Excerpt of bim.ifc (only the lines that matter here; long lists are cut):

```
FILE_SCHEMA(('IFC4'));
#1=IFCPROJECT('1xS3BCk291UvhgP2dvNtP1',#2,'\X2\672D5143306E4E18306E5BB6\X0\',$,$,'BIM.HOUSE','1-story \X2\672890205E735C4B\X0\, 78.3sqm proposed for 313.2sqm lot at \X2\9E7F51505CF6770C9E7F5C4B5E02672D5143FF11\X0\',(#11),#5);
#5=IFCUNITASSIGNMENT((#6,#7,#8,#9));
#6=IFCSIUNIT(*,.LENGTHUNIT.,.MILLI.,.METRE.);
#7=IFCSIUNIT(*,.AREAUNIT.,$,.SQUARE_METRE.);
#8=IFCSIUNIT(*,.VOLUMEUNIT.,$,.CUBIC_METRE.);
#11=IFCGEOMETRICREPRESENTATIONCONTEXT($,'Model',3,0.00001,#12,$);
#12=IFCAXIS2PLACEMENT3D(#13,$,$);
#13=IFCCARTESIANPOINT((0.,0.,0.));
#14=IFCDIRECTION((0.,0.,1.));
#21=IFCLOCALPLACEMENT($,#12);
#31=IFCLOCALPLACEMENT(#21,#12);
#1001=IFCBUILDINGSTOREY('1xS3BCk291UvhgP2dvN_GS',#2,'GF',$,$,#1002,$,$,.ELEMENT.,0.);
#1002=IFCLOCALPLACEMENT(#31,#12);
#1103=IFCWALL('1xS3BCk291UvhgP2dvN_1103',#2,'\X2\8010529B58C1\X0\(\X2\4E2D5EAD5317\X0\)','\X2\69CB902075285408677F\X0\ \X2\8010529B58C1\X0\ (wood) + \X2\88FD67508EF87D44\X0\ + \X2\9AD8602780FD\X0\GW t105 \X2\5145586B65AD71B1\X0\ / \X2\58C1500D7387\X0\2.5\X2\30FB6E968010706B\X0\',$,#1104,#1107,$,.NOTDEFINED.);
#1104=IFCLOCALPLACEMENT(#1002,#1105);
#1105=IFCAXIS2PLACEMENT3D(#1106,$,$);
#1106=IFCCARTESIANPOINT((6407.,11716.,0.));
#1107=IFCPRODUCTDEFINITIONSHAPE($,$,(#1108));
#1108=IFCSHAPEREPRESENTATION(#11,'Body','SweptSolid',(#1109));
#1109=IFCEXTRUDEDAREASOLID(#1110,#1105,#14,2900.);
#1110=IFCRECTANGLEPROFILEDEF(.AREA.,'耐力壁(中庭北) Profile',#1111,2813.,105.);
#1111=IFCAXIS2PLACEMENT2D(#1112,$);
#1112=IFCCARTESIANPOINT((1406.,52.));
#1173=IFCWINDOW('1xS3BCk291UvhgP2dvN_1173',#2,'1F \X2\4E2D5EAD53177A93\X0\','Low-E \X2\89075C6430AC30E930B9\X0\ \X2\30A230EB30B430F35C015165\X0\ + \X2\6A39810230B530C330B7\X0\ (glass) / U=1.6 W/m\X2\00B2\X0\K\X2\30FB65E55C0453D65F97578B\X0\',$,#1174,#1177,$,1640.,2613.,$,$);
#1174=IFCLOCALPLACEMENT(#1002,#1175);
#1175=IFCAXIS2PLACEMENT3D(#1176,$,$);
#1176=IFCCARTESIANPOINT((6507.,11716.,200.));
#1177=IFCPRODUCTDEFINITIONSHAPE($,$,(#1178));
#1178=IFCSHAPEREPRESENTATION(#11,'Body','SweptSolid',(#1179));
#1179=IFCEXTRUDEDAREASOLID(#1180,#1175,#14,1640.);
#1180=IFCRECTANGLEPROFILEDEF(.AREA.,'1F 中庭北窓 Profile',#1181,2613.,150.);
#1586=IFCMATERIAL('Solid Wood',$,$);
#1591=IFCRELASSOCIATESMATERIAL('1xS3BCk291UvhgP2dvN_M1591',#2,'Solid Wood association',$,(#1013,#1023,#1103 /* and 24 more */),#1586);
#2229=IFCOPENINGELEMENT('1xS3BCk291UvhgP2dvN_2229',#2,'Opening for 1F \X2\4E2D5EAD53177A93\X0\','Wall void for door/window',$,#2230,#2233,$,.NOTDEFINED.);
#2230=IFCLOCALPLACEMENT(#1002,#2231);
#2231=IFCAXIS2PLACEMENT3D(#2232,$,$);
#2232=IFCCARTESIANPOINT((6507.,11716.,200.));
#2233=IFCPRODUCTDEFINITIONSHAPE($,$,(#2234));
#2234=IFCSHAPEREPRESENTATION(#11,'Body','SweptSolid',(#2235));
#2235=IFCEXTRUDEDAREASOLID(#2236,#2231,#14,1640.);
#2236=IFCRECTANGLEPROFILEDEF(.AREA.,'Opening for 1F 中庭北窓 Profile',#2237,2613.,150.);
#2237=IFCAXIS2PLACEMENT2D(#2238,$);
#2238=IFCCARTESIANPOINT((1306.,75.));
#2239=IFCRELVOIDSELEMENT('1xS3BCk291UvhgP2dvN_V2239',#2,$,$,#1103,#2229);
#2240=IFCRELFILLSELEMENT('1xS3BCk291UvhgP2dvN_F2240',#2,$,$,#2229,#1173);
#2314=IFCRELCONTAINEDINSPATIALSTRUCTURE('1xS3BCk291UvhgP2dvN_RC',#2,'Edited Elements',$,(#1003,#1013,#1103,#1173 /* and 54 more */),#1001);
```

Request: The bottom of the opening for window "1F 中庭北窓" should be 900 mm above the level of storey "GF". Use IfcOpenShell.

```python
import numpy as np
import ifcopenshell
import ifcopenshell.api.geometry
import ifcopenshell.geom
import ifcopenshell.util.element
import ifcopenshell.util.placement
import ifcopenshell.util.shape
import ifcopenshell.util.unit

model = ifcopenshell.open("bim.ifc")
unit_scale = ifcopenshell.util.unit.calculate_unit_scale(model)

window = model.by_guid("1xS3BCk291UvhgP2dvN_1173")
opening = window.FillsVoids[0].RelatingOpeningElement
storey = ifcopenshell.util.element.get_container(window, ifc_class="IfcBuildingStorey")
level = ifcopenshell.util.placement.get_local_placement(storey.ObjectPlacement)[2, 3]

# The opening's origin need not be at the sill, so measure its lowest point.
shape = ifcopenshell.geom.create_shape(ifcopenshell.geom.settings(), opening)
bottom = ifcopenshell.util.shape.get_shape_bottom_elevation(shape, shape.geometry) / unit_scale
dz = level + 0.9 / unit_scale - bottom

shift = np.array([0.0, 0.0, dz])
# The window is not placed relative to its opening, so move both.
for product in (opening, window):
    matrix = ifcopenshell.util.placement.get_local_placement(product.ObjectPlacement)
    matrix[:3, 3] += shift
    ifcopenshell.api.geometry.edit_object_placement(model, product=product, matrix=matrix, is_si=False)

print(f"moved by {dz * unit_scale:+.3f} m")

model.write("bim_updated.ifc")
```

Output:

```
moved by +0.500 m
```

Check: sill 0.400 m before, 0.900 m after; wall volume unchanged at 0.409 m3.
